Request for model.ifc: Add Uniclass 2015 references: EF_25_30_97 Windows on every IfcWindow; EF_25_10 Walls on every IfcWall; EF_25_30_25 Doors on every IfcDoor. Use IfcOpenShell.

First a look at what the model holds.

```python
import ifcopenshell

model = ifcopenshell.open("model.ifc")
print(model.schema)
print("classifications:", [c.Name for c in model.by_type("IfcClassification")])
for ifc_class in ("IfcDoor", "IfcRoof", "IfcStair", "IfcWall", "IfcWindow"):
    print(ifc_class, len(model.by_type(ifc_class)))
```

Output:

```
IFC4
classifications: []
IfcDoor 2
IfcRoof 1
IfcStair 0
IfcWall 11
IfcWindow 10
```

```python
import ifcopenshell
import ifcopenshell.api.classification

model = ifcopenshell.open("model.ifc")

system = ifcopenshell.api.classification.add_classification(model, classification="Uniclass 2015")

codes = {
    "IfcWindow": ("EF_25_30_97", "Windows"),
    "IfcWall": ("EF_25_10", "Walls"),
    "IfcDoor": ("EF_25_30_25", "Doors"),
}
for ifc_class, (code, name) in codes.items():
    products = model.by_type(ifc_class)
    ifcopenshell.api.classification.add_reference(
        model, products=products, classification=system, identification=code, name=name
    )
    print(code, len(products))

model.write("model-out.ifc")
```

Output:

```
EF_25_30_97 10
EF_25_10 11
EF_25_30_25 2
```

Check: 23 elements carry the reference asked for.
